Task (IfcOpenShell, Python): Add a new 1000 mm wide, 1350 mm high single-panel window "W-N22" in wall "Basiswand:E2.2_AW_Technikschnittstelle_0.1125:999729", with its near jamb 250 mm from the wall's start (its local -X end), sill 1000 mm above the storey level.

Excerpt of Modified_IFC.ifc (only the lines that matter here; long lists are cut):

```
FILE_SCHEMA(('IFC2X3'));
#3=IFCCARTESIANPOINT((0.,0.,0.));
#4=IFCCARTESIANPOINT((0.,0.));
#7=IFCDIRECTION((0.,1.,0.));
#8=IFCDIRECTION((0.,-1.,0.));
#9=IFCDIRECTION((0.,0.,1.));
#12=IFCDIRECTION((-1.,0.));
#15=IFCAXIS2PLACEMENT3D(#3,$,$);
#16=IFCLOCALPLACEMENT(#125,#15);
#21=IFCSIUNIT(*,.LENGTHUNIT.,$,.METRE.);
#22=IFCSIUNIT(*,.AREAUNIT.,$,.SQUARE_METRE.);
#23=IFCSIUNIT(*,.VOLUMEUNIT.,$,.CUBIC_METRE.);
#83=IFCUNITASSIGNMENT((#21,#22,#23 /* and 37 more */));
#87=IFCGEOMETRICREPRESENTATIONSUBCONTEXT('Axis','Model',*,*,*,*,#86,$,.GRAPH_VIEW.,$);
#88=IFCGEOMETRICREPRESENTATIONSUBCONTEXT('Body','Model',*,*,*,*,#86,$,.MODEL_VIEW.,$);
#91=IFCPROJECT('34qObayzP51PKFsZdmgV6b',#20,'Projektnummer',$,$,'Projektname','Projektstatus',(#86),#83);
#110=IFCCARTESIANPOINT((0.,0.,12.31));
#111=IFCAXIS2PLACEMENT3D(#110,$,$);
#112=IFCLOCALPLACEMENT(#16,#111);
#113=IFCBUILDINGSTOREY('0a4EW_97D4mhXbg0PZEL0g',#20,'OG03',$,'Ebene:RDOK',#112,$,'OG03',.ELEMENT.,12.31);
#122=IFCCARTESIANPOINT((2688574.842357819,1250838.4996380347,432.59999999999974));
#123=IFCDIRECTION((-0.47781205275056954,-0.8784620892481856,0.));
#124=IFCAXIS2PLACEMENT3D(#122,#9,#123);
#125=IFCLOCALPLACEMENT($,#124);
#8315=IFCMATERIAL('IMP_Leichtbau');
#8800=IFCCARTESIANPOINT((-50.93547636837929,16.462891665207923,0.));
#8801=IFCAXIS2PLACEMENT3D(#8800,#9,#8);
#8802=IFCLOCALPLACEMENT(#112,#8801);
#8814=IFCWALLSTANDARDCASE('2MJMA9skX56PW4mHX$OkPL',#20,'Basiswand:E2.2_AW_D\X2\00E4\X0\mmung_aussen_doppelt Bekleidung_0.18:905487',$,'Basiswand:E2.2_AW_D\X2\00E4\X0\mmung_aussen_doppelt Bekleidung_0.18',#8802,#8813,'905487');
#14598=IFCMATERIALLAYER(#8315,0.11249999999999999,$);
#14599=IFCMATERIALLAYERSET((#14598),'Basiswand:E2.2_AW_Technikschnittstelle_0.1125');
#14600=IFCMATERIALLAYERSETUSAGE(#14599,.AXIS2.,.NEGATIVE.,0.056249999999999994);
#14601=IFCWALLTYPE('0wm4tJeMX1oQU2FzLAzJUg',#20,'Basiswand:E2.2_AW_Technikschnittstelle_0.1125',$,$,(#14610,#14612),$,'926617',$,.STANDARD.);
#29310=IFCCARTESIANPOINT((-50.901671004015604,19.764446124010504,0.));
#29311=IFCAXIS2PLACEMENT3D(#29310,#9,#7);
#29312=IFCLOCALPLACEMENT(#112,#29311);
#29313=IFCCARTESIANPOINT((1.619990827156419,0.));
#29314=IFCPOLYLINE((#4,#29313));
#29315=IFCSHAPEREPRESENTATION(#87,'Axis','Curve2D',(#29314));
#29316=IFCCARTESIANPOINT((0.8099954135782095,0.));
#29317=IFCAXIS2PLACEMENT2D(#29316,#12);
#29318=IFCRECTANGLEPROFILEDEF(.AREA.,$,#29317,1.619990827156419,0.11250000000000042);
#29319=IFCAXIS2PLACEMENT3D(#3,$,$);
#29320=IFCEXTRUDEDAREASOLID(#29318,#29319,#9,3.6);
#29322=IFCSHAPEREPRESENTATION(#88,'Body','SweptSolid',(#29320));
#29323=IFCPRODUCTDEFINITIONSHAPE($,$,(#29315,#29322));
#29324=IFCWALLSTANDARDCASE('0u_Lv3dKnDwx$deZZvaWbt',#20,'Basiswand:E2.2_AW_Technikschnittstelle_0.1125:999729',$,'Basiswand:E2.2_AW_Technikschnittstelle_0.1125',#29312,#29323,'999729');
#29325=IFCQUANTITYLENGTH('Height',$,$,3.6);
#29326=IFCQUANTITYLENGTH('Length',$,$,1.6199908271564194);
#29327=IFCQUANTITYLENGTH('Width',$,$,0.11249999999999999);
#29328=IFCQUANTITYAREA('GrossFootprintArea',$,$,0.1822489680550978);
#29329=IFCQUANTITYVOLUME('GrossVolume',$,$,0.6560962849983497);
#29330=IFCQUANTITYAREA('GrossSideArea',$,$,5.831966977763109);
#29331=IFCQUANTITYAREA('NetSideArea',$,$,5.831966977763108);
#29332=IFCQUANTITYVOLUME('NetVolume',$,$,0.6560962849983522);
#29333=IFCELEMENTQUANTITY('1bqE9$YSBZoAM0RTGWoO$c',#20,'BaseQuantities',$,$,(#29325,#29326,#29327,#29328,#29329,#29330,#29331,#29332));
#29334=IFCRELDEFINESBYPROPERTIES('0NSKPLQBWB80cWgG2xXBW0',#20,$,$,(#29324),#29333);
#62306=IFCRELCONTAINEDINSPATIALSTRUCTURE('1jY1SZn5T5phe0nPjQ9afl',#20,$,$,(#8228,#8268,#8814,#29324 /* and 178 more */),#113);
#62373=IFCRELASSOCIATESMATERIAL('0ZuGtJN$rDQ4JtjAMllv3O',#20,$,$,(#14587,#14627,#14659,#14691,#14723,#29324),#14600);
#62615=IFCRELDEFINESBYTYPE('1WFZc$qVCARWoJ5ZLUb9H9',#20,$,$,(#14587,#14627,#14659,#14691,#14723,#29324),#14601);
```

```python
import numpy as np
import ifcopenshell
import ifcopenshell.api.feature
import ifcopenshell.api.geometry
import ifcopenshell.api.pset
import ifcopenshell.api.root
import ifcopenshell.api.spatial
import ifcopenshell.api.type
import ifcopenshell.geom
import ifcopenshell.util.element
import ifcopenshell.util.placement
import ifcopenshell.util.representation
import ifcopenshell.util.shape
import ifcopenshell.util.unit

model = ifcopenshell.open("Modified_IFC.ifc")
unit_scale = ifcopenshell.util.unit.calculate_unit_scale(model)
area_scale = ifcopenshell.util.unit.calculate_unit_scale(model, "AREAUNIT")
volume_scale = ifcopenshell.util.unit.calculate_unit_scale(model, "VOLUMEUNIT")
settings = ifcopenshell.geom.settings()


def volume(element):
    """Net volume in cubic metres, openings subtracted."""
    shape = ifcopenshell.geom.create_shape(settings, element)
    return ifcopenshell.util.shape.get_volume(shape.geometry)


wall = model.by_id(29324)
storey = ifcopenshell.util.element.get_container(wall, ifc_class="IfcBuildingStorey")
context = ifcopenshell.util.representation.get_context(model, "Model", "Body", "MODEL_VIEW")
before = volume(wall)

width, height, from_end, sill = 1, 1.35, 0.25, 1  # metres

# The wall runs along its own X axis, and the end named is its -X end.
wall_shape = ifcopenshell.geom.create_shape(settings, wall)
x, y, z = ifcopenshell.util.shape.get_vertices(wall_shape.geometry).T
start = x.min() + from_end
face, thickness = float(y.min()), float(y.max() - y.min())
wall_matrix = ifcopenshell.util.placement.get_local_placement(wall.ObjectPlacement)
level = ifcopenshell.util.placement.get_local_placement(storey.ObjectPlacement)[2, 3]


def in_wall(x, y):
    """Placement at x, y metres in the wall's axes, at sill height."""
    matrix = wall_matrix.copy()
    matrix[:, 3] = wall_matrix @ np.array([x / unit_scale, y / unit_scale, 0.0, 1.0])
    matrix[2, 3] = level + sill / unit_scale
    return matrix


# Opening: a box that overshoots both wall faces by 50 mm.
opening = ifcopenshell.api.root.create_entity(model, ifc_class="IfcOpeningElement")
box = ifcopenshell.api.geometry.add_wall_representation(
    model, context=context, length=width, height=height, thickness=thickness + 0.1
)
ifcopenshell.api.geometry.assign_representation(model, product=opening, representation=box)
ifcopenshell.api.geometry.edit_object_placement(model, product=opening, matrix=in_wall(start, face - 0.05), is_si=False)
ifcopenshell.api.feature.add_feature(model, feature=opening, element=wall)

window = ifcopenshell.api.root.create_entity(model, ifc_class="IfcWindow", name="W-N22")
window.OverallWidth, window.OverallHeight = width / unit_scale, height / unit_scale
body = ifcopenshell.api.geometry.add_window_representation(
    model,
    context=context,
    overall_width=window.OverallWidth,
    overall_height=window.OverallHeight,
    partition_type="SINGLE_PANEL",
)
ifcopenshell.api.geometry.assign_representation(model, product=window, representation=body)
ifcopenshell.api.spatial.assign_container(model, products=[window], relating_structure=storey)
fills = ifcopenshell.api.feature.add_filling(model, opening=opening, element=window)
fills.OwnerHistory = window.OwnerHistory  # required in IFC2X3

# IFC2X3 keeps the operation on the window style.
style = ifcopenshell.api.root.create_entity(model, ifc_class="IfcWindowStyle", name="W-N22")
style.OperationType, style.ConstructionType = "SINGLE_PANEL", "NOTDEFINED"
style.ParameterTakesPrecedence = style.Sizeable = False
ifcopenshell.api.type.assign_type(model, related_objects=[window], relating_type=style)

# Centre the window in the wall's thickness.
ifcopenshell.api.geometry.edit_object_placement(model, product=window, matrix=in_wall(start, face), is_si=False)
window_shape = ifcopenshell.geom.create_shape(settings, window)
depth = ifcopenshell.util.shape.get_vertices(window_shape.geometry)[:, 1]
offset = face + thickness / 2 - (depth.min() + depth.max()) / 2
ifcopenshell.api.geometry.edit_object_placement(model, product=window, matrix=in_wall(start, offset), is_si=False)

after = volume(wall)

# Update the wall's stored quantities.
qto = model.by_id(ifcopenshell.util.element.get_pset(wall, "BaseQuantities", should_inherit=False)["id"])
ifcopenshell.api.pset.edit_qto(model, qto=qto, properties={
    "NetSideArea": after / thickness / area_scale,
    "NetVolume": after / volume_scale,
})

print(f"wall volume {before:.3f} -> {after:.3f} m3")

model.write("Modified_IFC_edited.ifc")
```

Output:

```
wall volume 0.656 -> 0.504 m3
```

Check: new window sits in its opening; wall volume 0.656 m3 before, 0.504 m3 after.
